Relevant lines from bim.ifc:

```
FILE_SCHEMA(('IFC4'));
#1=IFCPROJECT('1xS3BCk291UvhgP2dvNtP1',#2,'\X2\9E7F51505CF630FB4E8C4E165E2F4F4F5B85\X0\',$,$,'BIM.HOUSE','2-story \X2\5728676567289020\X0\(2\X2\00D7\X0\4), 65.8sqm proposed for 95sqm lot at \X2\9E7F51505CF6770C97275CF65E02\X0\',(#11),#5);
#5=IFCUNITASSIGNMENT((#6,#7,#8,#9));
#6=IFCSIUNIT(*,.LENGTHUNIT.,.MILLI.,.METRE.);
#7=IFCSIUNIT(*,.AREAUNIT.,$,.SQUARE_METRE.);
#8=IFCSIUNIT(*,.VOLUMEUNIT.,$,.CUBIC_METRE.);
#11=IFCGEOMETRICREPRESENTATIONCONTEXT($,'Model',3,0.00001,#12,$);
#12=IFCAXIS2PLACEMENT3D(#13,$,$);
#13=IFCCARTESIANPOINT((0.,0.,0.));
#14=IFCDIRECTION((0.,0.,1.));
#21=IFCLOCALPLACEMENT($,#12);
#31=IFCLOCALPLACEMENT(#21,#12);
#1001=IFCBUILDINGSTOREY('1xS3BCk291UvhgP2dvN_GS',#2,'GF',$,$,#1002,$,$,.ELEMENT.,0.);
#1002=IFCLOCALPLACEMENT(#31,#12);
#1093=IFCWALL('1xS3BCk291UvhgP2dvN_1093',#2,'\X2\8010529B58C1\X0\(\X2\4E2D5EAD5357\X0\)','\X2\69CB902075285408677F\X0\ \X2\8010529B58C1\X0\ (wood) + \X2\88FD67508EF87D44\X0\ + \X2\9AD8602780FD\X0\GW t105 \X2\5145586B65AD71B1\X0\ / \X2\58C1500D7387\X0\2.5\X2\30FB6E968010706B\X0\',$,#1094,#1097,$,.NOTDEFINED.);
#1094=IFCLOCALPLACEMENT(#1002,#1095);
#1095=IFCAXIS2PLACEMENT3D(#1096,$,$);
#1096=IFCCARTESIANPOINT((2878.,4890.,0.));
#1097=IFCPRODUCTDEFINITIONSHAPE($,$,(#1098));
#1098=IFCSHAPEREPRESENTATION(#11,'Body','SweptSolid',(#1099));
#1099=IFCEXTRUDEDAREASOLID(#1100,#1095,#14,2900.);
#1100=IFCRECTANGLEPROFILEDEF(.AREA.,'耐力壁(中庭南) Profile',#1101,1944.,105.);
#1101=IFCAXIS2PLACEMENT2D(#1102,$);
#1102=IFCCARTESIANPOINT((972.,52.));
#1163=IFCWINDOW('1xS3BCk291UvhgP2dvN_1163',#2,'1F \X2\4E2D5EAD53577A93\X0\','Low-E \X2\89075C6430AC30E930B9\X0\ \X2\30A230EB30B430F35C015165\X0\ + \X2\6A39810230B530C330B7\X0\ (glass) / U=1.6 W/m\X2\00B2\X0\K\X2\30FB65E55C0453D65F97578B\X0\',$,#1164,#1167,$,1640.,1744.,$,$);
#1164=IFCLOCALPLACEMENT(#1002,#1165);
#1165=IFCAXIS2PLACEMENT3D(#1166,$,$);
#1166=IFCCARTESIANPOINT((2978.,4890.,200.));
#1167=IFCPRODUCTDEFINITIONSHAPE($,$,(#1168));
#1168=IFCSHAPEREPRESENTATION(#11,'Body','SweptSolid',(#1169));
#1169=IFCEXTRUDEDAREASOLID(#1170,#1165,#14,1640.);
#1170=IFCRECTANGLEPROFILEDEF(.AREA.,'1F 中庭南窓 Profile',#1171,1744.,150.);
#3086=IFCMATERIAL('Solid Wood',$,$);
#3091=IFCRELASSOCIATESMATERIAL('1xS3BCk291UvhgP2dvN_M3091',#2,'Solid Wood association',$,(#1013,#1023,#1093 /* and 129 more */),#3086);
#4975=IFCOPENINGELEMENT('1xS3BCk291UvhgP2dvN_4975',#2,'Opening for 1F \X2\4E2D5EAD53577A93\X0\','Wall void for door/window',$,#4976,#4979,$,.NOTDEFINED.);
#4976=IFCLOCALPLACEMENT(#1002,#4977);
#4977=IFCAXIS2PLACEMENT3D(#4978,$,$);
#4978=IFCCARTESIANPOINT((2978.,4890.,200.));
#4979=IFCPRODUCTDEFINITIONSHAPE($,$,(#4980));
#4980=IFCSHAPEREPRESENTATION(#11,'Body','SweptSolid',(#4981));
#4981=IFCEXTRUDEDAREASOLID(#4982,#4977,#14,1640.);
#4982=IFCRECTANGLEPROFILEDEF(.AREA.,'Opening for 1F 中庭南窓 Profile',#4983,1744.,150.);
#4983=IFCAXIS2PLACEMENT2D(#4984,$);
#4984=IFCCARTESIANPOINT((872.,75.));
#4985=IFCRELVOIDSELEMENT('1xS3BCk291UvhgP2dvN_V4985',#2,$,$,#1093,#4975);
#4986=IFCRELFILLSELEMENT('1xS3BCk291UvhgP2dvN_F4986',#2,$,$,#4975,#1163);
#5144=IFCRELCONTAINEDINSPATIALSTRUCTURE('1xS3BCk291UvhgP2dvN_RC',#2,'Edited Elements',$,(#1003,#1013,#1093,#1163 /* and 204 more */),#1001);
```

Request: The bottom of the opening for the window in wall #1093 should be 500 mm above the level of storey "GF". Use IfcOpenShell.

```python
import numpy as np
import ifcopenshell
import ifcopenshell.api.geometry
import ifcopenshell.geom
import ifcopenshell.util.element
import ifcopenshell.util.placement
import ifcopenshell.util.shape
import ifcopenshell.util.unit

model = ifcopenshell.open("bim.ifc")
unit_scale = ifcopenshell.util.unit.calculate_unit_scale(model)

window = model.by_guid("1xS3BCk291UvhgP2dvN_1163")
opening = window.FillsVoids[0].RelatingOpeningElement
storey = ifcopenshell.util.element.get_container(window, ifc_class="IfcBuildingStorey")
level = ifcopenshell.util.placement.get_local_placement(storey.ObjectPlacement)[2, 3]

# The opening's origin need not be at the sill, so measure its lowest point.
shape = ifcopenshell.geom.create_shape(ifcopenshell.geom.settings(), opening)
bottom = ifcopenshell.util.shape.get_shape_bottom_elevation(shape, shape.geometry) / unit_scale
dz = level + 0.5 / unit_scale - bottom

shift = np.array([0.0, 0.0, dz])
# The window is not placed relative to its opening, so move both.
for product in (opening, window):
    matrix = ifcopenshell.util.placement.get_local_placement(product.ObjectPlacement)
    matrix[:3, 3] += shift
    ifcopenshell.api.geometry.edit_object_placement(model, product=product, matrix=matrix, is_si=False)

print(f"moved by {dz * unit_scale:+.3f} m")

model.write("bim_rev.ifc")
```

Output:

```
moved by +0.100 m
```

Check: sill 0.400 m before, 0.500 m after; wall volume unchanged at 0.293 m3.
